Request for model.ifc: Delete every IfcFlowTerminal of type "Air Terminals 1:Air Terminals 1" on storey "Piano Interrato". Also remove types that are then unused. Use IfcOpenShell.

First a look at what the model holds.

```python
import ifcopenshell
import ifcopenshell.util.element

model = ifcopenshell.open("model.ifc")
print(model.schema)
storey = next(s for s in model.by_type("IfcBuildingStorey") if s.Name == "Piano Interrato")
terminals = [e for e in ifcopenshell.util.element.get_decomposition(storey) if e.is_a("IfcFlowTerminal")]
seen = {}
for e in terminals:
    element_type = ifcopenshell.util.element.get_type(e)
    name = element_type.Name if element_type not in (None, e) else None
    seen[name] = seen.get(name, 0) + 1
for name, count in sorted(seen.items(), key=str):
    print(count, "x", name)
```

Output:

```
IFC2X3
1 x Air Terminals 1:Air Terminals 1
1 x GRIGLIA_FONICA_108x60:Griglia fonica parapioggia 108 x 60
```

```python
import ifcopenshell
import ifcopenshell.api.root
import ifcopenshell.util.element

model = ifcopenshell.open("model.ifc")

storey = next(s for s in model.by_type("IfcBuildingStorey") if s.Name == "Piano Interrato")
terminals = [e for e in ifcopenshell.util.element.get_decomposition(storey) if e.is_a("IfcFlowTerminal")]
targets = [e for e in terminals if (t := ifcopenshell.util.element.get_type(e)) not in (None, e) and t.Name == "Air Terminals 1:Air Terminals 1"]
types = {ifcopenshell.util.element.get_type(e) for e in targets} - {None, *targets}

for e in targets:
    ifcopenshell.api.root.remove_product(model, product=e)
print(len(targets), "removed")

unused = [t for t in types if not ifcopenshell.util.element.get_types(t)]
for t in unused:
    ifcopenshell.api.root.remove_product(model, product=t)
print(len(unused), "unused types removed")

model.write("model_edited.ifc")
```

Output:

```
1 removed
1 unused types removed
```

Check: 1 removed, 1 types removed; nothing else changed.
